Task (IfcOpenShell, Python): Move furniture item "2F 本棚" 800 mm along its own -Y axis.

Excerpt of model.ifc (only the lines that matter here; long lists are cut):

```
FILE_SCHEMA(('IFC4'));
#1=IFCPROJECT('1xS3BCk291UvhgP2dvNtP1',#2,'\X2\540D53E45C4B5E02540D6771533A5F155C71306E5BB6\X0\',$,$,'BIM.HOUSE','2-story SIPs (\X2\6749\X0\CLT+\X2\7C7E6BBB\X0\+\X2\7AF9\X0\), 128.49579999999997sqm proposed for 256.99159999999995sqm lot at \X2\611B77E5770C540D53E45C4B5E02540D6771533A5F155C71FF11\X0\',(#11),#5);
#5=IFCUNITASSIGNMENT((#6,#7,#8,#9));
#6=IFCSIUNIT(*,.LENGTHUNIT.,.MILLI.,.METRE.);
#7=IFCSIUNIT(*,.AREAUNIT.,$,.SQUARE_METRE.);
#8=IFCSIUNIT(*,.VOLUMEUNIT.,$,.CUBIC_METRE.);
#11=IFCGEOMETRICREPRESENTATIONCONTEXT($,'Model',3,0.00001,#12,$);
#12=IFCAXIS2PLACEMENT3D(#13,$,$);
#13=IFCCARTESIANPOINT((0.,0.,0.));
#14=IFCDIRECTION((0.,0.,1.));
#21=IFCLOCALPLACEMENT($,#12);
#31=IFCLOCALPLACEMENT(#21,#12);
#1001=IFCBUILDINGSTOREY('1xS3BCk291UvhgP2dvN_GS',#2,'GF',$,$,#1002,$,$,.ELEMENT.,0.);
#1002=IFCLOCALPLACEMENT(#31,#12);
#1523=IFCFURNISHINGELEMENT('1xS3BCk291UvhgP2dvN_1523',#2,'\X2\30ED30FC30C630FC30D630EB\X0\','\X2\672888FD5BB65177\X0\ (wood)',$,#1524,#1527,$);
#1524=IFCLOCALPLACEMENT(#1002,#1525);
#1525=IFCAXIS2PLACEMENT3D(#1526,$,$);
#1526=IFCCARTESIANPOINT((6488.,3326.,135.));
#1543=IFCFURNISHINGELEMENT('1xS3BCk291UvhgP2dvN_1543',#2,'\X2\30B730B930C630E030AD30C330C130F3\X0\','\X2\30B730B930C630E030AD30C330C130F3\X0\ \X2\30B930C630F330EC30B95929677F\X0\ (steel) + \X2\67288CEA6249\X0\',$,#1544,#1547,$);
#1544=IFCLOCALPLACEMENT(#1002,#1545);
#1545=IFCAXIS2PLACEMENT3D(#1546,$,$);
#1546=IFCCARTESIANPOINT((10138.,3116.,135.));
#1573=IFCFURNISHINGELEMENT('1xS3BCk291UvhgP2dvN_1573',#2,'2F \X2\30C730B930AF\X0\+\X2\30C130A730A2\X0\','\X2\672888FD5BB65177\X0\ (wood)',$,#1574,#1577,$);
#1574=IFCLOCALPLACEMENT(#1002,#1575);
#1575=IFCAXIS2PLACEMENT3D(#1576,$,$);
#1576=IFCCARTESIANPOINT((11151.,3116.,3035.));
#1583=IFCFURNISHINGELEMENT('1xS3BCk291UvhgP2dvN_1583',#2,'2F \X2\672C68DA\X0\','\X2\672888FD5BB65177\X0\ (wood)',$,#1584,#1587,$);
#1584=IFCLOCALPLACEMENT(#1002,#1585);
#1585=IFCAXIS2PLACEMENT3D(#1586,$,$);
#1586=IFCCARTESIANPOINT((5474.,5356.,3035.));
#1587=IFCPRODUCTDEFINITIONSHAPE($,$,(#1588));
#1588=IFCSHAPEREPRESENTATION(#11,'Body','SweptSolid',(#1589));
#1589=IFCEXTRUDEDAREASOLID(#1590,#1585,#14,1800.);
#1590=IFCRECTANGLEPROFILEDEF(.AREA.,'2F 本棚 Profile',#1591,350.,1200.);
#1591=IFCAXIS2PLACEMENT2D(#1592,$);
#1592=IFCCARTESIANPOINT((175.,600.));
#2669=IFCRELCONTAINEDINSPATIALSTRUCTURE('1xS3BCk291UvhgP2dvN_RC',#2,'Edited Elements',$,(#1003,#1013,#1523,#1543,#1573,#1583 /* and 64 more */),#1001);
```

```python
import ifcopenshell
import ifcopenshell.api.geometry
import ifcopenshell.util.placement

model = ifcopenshell.open("model.ifc")

item = model.by_id(1583)
matrix = ifcopenshell.util.placement.get_local_placement(item.ObjectPlacement)
matrix[:3, 3] -= matrix[:3, 1] * 800.0
ifcopenshell.api.geometry.edit_object_placement(model, product=item, matrix=matrix, is_si=False)

print(ifcopenshell.util.placement.get_local_placement(item.ObjectPlacement).round(3) + 0.0)

model.write("model_edited.ifc")
```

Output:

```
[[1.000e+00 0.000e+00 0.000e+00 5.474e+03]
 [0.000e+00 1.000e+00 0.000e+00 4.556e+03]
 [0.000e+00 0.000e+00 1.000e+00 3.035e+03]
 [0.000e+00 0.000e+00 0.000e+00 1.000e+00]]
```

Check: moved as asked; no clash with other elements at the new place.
